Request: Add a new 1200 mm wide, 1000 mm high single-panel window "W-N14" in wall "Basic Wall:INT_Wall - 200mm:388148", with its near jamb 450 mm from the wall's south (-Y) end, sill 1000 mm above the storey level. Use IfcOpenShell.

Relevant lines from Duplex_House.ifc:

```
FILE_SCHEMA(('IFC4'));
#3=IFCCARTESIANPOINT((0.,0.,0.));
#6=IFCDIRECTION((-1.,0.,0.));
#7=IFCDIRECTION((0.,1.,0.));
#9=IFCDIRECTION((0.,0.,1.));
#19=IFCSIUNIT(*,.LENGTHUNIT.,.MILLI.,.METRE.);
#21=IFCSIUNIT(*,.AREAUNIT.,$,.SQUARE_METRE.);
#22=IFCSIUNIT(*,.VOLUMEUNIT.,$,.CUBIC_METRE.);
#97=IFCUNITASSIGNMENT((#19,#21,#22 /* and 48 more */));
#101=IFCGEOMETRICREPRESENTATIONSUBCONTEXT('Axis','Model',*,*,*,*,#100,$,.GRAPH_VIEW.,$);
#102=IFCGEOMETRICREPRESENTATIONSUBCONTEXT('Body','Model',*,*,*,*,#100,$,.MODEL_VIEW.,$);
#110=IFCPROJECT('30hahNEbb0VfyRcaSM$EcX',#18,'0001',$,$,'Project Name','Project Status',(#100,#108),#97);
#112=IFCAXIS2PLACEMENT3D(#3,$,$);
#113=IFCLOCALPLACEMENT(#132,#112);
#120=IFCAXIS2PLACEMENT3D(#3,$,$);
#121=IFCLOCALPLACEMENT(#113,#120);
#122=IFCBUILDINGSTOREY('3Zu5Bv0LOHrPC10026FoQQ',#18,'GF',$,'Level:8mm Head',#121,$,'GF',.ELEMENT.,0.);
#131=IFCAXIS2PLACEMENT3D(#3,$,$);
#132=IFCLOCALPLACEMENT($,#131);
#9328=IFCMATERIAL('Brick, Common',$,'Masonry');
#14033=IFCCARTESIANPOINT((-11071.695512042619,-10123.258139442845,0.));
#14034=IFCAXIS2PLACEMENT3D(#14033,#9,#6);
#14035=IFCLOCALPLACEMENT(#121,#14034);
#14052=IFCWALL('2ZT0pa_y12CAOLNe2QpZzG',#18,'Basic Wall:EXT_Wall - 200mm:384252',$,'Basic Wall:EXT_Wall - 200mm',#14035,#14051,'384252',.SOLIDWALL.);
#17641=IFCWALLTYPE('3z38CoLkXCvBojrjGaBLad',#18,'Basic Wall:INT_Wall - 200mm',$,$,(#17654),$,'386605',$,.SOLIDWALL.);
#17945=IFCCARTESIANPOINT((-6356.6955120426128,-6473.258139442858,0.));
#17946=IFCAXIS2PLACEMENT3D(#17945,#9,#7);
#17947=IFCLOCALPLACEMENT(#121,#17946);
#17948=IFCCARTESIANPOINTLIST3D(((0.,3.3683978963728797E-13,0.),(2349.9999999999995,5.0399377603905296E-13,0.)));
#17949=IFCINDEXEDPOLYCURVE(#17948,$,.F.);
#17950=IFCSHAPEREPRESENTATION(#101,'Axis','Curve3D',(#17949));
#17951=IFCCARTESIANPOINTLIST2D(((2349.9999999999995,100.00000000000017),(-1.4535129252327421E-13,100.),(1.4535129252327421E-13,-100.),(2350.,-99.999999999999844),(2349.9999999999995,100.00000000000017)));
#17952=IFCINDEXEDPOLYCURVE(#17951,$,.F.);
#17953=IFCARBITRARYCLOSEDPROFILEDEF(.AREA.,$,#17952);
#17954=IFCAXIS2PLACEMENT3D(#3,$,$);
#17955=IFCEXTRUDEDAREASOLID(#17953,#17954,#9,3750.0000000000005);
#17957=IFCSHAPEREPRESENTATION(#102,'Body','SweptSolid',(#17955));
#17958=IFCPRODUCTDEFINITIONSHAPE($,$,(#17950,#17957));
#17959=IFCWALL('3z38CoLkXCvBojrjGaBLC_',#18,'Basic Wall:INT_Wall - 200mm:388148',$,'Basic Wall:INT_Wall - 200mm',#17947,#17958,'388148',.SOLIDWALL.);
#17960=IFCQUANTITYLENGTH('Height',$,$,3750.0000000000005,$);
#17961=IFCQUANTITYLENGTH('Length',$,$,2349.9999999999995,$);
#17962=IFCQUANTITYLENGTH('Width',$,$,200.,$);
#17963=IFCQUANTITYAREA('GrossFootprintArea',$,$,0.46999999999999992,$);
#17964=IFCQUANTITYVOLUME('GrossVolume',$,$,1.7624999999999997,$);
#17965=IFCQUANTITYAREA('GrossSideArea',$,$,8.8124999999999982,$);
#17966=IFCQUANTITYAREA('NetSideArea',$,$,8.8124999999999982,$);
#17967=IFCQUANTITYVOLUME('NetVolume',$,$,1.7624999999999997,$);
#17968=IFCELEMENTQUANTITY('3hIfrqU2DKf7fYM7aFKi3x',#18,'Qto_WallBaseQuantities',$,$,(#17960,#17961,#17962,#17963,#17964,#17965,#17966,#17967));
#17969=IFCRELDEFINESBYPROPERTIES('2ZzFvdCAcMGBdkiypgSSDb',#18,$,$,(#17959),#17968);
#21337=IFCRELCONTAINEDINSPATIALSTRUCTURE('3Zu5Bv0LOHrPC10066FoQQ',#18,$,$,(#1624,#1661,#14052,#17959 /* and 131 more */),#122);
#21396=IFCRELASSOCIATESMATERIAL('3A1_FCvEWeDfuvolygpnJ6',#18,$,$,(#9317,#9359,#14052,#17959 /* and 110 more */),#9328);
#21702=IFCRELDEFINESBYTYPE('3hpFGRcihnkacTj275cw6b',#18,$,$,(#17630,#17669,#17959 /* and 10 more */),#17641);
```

```python
import numpy as np
import ifcopenshell
import ifcopenshell.api.feature
import ifcopenshell.api.geometry
import ifcopenshell.api.pset
import ifcopenshell.api.root
import ifcopenshell.api.spatial
import ifcopenshell.geom
import ifcopenshell.util.element
import ifcopenshell.util.placement
import ifcopenshell.util.representation
import ifcopenshell.util.shape
import ifcopenshell.util.unit

model = ifcopenshell.open("Duplex_House.ifc")
unit_scale = ifcopenshell.util.unit.calculate_unit_scale(model)
area_scale = ifcopenshell.util.unit.calculate_unit_scale(model, "AREAUNIT")
volume_scale = ifcopenshell.util.unit.calculate_unit_scale(model, "VOLUMEUNIT")
settings = ifcopenshell.geom.settings()


def volume(element):
    """Net volume in cubic metres, openings subtracted."""
    shape = ifcopenshell.geom.create_shape(settings, element)
    return ifcopenshell.util.shape.get_volume(shape.geometry)


wall = model.by_guid("3z38CoLkXCvBojrjGaBLC_")
storey = ifcopenshell.util.element.get_container(wall, ifc_class="IfcBuildingStorey")
context = ifcopenshell.util.representation.get_context(model, "Model", "Body", "MODEL_VIEW")
before = volume(wall)

width, height, from_end, sill = 1.2, 1, 0.45, 1  # metres

# The wall runs along its own X axis, and the end named is its -X end.
wall_shape = ifcopenshell.geom.create_shape(settings, wall)
x, y, z = ifcopenshell.util.shape.get_vertices(wall_shape.geometry).T
start = x.min() + from_end
face, thickness = float(y.min()), float(y.max() - y.min())
wall_matrix = ifcopenshell.util.placement.get_local_placement(wall.ObjectPlacement)
level = ifcopenshell.util.placement.get_local_placement(storey.ObjectPlacement)[2, 3]


def in_wall(x, y):
    """Placement at x, y metres in the wall's axes, at sill height."""
    matrix = wall_matrix.copy()
    matrix[:, 3] = wall_matrix @ np.array([x / unit_scale, y / unit_scale, 0.0, 1.0])
    matrix[2, 3] = level + sill / unit_scale
    return matrix


# Opening: a box that overshoots both wall faces by 50 mm.
opening = ifcopenshell.api.root.create_entity(model, ifc_class="IfcOpeningElement", predefined_type="OPENING")
box = ifcopenshell.api.geometry.add_wall_representation(
    model, context=context, length=width, height=height, thickness=thickness + 0.1
)
ifcopenshell.api.geometry.assign_representation(model, product=opening, representation=box)
ifcopenshell.api.geometry.edit_object_placement(model, product=opening, matrix=in_wall(start, face - 0.05), is_si=False)
ifcopenshell.api.feature.add_feature(model, feature=opening, element=wall)

window = ifcopenshell.api.root.create_entity(model, ifc_class="IfcWindow", name="W-N14", predefined_type="WINDOW")
window.OverallWidth, window.OverallHeight = width / unit_scale, height / unit_scale
window.PartitioningType = "SINGLE_PANEL"
body = ifcopenshell.api.geometry.add_window_representation(
    model,
    context=context,
    overall_width=window.OverallWidth,
    overall_height=window.OverallHeight,
    partition_type="SINGLE_PANEL",
)
ifcopenshell.api.geometry.assign_representation(model, product=window, representation=body)
ifcopenshell.api.spatial.assign_container(model, products=[window], relating_structure=storey)
ifcopenshell.api.feature.add_filling(model, opening=opening, element=window)

# Centre the window in the wall's thickness.
ifcopenshell.api.geometry.edit_object_placement(model, product=window, matrix=in_wall(start, face), is_si=False)
window_shape = ifcopenshell.geom.create_shape(settings, window)
depth = ifcopenshell.util.shape.get_vertices(window_shape.geometry)[:, 1]
offset = face + thickness / 2 - (depth.min() + depth.max()) / 2
ifcopenshell.api.geometry.edit_object_placement(model, product=window, matrix=in_wall(start, offset), is_si=False)

after = volume(wall)

# Update the wall's stored quantities.
qto = model.by_id(ifcopenshell.util.element.get_pset(wall, "Qto_WallBaseQuantities", should_inherit=False)["id"])
ifcopenshell.api.pset.edit_qto(model, qto=qto, properties={
    "NetSideArea": after / thickness / area_scale,
    "NetVolume": after / volume_scale,
})

print(f"wall volume {before:.3f} -> {after:.3f} m3")

model.write("Duplex_House_rev.ifc")
```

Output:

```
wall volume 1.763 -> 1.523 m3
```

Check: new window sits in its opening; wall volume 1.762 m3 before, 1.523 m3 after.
